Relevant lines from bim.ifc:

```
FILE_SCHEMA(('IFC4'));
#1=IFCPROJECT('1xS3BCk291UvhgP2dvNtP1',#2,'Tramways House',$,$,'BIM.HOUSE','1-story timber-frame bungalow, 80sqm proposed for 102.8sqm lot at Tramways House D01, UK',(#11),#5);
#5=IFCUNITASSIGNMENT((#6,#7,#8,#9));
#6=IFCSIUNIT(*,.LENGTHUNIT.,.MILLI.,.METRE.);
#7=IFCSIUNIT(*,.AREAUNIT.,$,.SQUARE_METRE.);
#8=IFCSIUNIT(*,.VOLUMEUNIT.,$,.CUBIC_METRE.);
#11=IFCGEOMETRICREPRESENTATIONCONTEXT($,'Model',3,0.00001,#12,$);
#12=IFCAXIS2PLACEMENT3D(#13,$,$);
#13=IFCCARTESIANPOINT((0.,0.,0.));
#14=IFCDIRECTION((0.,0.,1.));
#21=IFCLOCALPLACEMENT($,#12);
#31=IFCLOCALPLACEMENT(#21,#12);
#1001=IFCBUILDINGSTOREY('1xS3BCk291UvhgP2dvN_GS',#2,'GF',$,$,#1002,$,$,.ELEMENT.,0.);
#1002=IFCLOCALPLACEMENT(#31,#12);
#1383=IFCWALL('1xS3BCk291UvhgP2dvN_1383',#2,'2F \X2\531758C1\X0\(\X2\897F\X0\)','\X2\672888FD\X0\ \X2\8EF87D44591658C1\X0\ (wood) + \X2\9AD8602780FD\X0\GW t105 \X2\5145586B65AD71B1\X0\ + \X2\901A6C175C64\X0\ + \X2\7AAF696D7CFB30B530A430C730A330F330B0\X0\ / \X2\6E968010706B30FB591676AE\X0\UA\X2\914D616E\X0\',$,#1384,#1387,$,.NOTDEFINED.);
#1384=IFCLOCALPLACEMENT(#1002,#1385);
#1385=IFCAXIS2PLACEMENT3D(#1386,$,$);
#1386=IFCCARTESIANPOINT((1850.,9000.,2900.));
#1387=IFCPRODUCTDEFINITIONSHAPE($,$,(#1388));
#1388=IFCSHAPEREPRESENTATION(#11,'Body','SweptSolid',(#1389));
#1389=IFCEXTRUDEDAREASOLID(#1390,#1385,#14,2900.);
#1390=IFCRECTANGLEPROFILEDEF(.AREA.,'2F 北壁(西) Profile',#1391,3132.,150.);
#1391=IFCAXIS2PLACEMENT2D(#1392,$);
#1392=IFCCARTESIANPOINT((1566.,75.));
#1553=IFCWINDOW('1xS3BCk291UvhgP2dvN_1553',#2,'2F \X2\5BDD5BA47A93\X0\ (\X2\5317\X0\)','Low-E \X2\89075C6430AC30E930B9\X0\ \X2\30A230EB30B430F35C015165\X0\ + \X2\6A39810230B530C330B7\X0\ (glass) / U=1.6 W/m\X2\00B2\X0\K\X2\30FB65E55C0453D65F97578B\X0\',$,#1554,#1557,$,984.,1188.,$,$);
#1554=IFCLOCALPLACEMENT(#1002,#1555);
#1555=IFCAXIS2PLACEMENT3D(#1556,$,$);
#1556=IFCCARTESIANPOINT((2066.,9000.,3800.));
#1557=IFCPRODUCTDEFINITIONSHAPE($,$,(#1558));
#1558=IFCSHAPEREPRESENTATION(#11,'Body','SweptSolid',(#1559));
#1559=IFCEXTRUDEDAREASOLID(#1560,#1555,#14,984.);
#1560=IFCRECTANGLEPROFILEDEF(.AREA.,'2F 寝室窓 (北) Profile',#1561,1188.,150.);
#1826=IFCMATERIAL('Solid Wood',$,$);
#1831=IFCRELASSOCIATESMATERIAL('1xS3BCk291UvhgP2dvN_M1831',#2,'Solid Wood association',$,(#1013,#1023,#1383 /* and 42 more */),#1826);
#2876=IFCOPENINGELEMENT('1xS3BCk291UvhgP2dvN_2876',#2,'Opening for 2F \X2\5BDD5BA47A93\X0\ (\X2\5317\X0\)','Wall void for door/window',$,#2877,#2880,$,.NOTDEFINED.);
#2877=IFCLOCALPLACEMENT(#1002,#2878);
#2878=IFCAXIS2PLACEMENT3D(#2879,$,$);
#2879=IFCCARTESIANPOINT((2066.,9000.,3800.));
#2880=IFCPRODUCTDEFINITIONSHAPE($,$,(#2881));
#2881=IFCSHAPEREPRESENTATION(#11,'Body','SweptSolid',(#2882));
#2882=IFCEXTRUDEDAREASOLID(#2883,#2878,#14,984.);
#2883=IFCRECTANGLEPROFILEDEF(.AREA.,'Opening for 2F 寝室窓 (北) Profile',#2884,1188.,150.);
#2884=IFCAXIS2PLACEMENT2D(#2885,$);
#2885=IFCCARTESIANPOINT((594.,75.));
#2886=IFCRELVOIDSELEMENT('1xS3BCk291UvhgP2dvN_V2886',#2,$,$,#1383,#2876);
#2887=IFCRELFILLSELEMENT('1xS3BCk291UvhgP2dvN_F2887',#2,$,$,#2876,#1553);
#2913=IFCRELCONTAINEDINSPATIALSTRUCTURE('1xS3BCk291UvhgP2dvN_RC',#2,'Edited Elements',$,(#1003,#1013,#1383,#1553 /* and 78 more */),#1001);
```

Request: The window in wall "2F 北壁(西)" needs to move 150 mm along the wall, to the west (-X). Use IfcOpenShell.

```python
import ifcopenshell
import ifcopenshell.api.geometry
import ifcopenshell.util.placement

model = ifcopenshell.open("bim.ifc")

window = model.by_id(1553)
opening = window.FillsVoids[0].RelatingOpeningElement
wall = opening.VoidsElements[0].RelatingBuildingElement

wall_matrix = ifcopenshell.util.placement.get_local_placement(wall.ObjectPlacement)
shift = wall_matrix[:3, 0] * -150.0
before = ifcopenshell.util.placement.get_local_placement(window.ObjectPlacement)[:3, 3].copy()

# The window is not placed relative to its opening, so move both.
for product in (opening, window):
    matrix = ifcopenshell.util.placement.get_local_placement(product.ObjectPlacement)
    matrix[:3, 3] += shift
    ifcopenshell.api.geometry.edit_object_placement(model, product=product, matrix=matrix, is_si=False)

after = ifcopenshell.util.placement.get_local_placement(window.ObjectPlacement)[:3, 3]
print("window moved by", (after - before).round(3) + 0.0)

model.write("bim_edited.ifc")
```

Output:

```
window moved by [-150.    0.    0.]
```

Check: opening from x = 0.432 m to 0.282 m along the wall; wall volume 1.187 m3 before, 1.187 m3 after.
